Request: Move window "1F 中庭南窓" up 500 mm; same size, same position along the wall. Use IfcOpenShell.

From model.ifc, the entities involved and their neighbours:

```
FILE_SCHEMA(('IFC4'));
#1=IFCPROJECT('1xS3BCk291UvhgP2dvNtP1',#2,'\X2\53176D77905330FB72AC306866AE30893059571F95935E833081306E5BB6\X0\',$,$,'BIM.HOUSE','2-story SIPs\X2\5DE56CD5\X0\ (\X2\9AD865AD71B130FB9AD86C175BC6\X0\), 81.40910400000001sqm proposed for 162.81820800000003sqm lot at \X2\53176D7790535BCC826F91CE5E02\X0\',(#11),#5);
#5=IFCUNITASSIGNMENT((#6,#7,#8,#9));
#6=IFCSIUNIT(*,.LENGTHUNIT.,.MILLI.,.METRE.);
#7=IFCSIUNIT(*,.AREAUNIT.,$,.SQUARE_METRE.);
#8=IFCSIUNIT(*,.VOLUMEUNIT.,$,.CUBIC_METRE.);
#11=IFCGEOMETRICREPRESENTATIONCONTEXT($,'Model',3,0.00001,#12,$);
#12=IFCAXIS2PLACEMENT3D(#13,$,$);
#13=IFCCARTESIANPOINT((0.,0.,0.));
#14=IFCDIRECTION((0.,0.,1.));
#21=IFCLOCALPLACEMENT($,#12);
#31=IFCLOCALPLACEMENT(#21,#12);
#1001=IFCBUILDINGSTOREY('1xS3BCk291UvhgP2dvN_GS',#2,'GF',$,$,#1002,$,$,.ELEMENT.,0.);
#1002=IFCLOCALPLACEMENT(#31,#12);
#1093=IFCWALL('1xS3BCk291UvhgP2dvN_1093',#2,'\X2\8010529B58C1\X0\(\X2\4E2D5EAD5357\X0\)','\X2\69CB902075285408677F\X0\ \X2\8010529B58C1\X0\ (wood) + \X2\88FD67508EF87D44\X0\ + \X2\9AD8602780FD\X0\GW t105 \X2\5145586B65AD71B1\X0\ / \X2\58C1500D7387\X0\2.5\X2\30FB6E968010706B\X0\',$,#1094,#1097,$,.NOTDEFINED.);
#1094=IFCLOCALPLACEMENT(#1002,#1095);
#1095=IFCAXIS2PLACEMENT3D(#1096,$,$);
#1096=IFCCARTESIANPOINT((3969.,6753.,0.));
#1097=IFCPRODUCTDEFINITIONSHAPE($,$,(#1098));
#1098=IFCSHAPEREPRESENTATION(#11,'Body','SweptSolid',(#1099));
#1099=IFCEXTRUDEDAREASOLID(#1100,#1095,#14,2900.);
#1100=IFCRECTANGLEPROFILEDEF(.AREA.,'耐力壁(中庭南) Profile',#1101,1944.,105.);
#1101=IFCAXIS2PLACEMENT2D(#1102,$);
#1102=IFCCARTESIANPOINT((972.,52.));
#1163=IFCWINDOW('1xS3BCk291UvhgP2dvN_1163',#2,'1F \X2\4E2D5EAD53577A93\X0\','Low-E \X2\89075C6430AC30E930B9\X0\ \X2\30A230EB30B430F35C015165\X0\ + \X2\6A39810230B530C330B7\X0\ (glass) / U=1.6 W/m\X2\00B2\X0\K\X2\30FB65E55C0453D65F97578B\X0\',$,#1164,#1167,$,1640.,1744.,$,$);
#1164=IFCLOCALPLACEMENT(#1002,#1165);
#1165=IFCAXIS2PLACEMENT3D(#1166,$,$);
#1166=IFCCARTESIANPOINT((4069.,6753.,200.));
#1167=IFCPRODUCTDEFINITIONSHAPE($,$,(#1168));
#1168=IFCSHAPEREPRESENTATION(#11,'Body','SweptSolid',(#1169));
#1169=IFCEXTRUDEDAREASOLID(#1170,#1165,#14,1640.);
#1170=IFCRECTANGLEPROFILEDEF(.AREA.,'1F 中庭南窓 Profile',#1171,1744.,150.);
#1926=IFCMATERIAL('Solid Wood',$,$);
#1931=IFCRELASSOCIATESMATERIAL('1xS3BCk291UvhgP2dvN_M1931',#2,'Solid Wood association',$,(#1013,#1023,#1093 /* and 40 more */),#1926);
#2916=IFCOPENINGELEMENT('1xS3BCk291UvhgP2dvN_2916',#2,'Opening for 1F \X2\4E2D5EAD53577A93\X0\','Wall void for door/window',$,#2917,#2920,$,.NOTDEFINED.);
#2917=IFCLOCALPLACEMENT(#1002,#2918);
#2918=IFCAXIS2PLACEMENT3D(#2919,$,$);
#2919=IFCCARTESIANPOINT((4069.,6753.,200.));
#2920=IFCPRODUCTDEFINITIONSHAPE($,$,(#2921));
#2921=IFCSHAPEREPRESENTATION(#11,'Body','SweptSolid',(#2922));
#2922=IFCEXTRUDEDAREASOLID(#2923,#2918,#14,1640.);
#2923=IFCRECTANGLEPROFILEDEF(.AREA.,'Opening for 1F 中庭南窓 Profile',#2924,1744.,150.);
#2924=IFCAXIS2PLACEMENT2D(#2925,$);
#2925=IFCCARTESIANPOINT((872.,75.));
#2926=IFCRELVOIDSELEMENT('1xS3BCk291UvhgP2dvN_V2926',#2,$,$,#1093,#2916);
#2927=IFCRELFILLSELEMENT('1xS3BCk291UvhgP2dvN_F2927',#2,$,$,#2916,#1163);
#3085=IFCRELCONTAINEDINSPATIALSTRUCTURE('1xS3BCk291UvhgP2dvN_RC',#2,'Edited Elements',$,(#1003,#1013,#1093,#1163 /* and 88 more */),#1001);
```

```python
import numpy as np
import ifcopenshell
import ifcopenshell.api.geometry
import ifcopenshell.util.placement
import ifcopenshell.util.unit

model = ifcopenshell.open("model.ifc")
unit_scale = ifcopenshell.util.unit.calculate_unit_scale(model)

window = model.by_id(1163)
opening = window.FillsVoids[0].RelatingOpeningElement
dz = 0.5 / unit_scale

shift = np.array([0.0, 0.0, dz])
# The window is not placed relative to its opening, so move both.
for product in (opening, window):
    matrix = ifcopenshell.util.placement.get_local_placement(product.ObjectPlacement)
    matrix[:3, 3] += shift
    ifcopenshell.api.geometry.edit_object_placement(model, product=product, matrix=matrix, is_si=False)

print(f"moved by {dz * unit_scale:+.3f} m")

model.write("model_v2.ifc")
```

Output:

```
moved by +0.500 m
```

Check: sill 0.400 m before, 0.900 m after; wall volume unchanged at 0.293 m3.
